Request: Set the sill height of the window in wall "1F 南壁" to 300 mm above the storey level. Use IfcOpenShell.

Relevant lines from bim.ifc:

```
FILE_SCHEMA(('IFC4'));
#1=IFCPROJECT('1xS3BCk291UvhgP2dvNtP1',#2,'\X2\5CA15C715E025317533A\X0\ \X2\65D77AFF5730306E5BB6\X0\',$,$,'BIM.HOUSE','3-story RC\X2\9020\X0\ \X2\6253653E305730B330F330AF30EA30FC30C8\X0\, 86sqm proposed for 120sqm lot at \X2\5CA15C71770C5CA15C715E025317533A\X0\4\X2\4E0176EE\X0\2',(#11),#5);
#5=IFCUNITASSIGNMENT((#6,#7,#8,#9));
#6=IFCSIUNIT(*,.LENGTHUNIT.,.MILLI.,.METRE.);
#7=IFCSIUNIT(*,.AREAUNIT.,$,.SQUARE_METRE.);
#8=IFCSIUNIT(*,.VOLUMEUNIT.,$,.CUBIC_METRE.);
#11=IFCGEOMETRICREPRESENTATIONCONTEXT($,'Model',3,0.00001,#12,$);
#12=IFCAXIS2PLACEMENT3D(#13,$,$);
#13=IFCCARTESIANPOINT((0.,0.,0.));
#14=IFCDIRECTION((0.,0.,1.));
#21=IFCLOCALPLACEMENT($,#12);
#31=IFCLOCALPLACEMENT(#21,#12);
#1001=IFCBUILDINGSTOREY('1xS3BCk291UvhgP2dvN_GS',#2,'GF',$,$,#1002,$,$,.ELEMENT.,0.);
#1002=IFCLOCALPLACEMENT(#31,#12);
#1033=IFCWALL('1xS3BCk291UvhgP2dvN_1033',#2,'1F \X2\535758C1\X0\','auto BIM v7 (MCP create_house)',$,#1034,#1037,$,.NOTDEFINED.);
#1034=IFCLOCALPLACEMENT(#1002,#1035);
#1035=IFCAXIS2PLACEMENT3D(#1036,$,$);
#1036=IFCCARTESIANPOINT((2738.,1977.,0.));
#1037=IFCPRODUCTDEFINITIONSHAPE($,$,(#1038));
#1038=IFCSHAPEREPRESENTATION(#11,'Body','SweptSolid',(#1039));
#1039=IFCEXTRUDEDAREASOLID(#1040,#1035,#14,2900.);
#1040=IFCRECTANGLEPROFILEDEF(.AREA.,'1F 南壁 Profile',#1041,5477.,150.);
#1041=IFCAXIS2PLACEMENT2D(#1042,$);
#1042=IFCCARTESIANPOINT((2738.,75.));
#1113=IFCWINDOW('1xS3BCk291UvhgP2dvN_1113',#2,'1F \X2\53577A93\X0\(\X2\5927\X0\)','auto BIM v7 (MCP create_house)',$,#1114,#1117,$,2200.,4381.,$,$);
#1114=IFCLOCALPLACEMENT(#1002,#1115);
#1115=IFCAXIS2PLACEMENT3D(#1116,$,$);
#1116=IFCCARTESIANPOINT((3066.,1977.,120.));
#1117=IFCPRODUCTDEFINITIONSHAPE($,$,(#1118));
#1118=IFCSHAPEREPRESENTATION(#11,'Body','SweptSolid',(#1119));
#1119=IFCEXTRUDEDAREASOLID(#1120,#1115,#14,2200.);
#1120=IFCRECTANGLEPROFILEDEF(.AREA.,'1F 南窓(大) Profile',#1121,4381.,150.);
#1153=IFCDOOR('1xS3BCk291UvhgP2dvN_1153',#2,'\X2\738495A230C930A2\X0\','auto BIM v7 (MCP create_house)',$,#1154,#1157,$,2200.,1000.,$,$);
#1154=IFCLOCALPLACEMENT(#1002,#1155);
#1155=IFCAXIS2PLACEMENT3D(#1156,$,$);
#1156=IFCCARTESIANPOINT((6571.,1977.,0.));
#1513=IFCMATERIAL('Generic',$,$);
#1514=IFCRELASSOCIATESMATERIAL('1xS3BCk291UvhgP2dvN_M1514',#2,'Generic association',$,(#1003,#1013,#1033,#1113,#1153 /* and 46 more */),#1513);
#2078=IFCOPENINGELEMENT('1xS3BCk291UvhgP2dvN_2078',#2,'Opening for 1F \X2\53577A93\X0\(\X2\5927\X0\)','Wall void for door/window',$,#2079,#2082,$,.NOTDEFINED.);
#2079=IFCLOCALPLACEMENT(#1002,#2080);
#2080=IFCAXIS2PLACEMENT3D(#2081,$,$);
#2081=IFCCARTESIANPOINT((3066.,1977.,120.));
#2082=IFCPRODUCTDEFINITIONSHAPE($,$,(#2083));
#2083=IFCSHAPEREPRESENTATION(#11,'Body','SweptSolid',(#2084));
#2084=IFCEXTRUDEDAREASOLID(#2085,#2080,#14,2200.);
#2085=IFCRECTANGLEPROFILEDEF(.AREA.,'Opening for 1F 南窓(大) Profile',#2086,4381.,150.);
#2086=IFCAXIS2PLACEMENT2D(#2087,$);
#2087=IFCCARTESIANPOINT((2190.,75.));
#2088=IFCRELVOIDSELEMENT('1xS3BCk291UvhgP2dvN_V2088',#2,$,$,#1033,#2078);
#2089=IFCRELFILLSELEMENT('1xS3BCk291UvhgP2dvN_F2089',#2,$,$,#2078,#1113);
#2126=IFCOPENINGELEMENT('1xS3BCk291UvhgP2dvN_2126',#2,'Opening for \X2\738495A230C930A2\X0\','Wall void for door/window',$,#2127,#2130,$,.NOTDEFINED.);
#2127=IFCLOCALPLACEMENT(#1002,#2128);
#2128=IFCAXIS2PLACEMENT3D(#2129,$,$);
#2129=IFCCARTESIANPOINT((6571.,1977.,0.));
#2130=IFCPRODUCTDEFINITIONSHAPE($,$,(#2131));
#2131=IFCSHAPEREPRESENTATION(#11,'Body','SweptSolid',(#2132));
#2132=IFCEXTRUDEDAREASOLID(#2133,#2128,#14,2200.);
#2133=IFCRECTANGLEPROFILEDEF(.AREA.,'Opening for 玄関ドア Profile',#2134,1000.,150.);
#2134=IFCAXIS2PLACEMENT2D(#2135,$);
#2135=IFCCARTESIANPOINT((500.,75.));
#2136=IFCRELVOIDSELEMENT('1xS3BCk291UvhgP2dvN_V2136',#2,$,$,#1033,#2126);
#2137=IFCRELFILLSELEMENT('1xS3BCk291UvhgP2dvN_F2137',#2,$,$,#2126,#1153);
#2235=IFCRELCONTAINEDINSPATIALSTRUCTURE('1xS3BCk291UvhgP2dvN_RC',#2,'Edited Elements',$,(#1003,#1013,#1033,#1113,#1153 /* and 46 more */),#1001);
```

```python
import numpy as np
import ifcopenshell
import ifcopenshell.api.geometry
import ifcopenshell.geom
import ifcopenshell.util.element
import ifcopenshell.util.placement
import ifcopenshell.util.shape
import ifcopenshell.util.unit

model = ifcopenshell.open("bim.ifc")
unit_scale = ifcopenshell.util.unit.calculate_unit_scale(model)

window = model.by_guid("1xS3BCk291UvhgP2dvN_1113")
opening = window.FillsVoids[0].RelatingOpeningElement
storey = ifcopenshell.util.element.get_container(window, ifc_class="IfcBuildingStorey")
level = ifcopenshell.util.placement.get_local_placement(storey.ObjectPlacement)[2, 3]

# The opening's origin need not be at the sill, so measure its lowest point.
shape = ifcopenshell.geom.create_shape(ifcopenshell.geom.settings(), opening)
bottom = ifcopenshell.util.shape.get_shape_bottom_elevation(shape, shape.geometry) / unit_scale
dz = level + 0.3 / unit_scale - bottom

shift = np.array([0.0, 0.0, dz])
# The window is not placed relative to its opening, so move both.
for product in (opening, window):
    matrix = ifcopenshell.util.placement.get_local_placement(product.ObjectPlacement)
    matrix[:3, 3] += shift
    ifcopenshell.api.geometry.edit_object_placement(model, product=product, matrix=matrix, is_si=False)

print(f"moved by {dz * unit_scale:+.3f} m")

model.write("bim-out.ifc")
```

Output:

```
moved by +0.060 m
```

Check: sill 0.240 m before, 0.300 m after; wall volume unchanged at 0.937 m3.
